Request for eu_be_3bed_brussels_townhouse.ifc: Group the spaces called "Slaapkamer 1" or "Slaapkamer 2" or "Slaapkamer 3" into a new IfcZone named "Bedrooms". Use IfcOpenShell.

First a look at what the model holds.

```python
import ifcopenshell

model = ifcopenshell.open("eu_be_3bed_brussels_townhouse.ifc")
print(model.schema)
seen = {}
for space in model.by_type("IfcSpace"):
    seen[space.LongName] = seen.get(space.LongName, 0) + 1
for name, count in sorted(seen.items(), key=str):
    print(count, "x", name)
print("zones:", [z.Name for z in model.by_type("IfcZone")][:20])
```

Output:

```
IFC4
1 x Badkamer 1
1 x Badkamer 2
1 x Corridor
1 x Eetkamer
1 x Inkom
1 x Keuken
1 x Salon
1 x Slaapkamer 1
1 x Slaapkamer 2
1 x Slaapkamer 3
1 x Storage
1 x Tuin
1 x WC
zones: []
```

```python
import ifcopenshell
import ifcopenshell.api.group
import ifcopenshell.api.root

model = ifcopenshell.open("eu_be_3bed_brussels_townhouse.ifc")

names = {"Slaapkamer 1", "Slaapkamer 2", "Slaapkamer 3"}
spaces = [s for s in model.by_type("IfcSpace") if s.LongName in names]

zone = ifcopenshell.api.root.create_entity(model, ifc_class="IfcZone", name="Bedrooms")
ifcopenshell.api.group.assign_group(model, products=spaces, group=zone)
print(len(spaces), "spaces in", zone.Name)

model.write("eu_be_3bed_brussels_townhouse_edited.ifc")
```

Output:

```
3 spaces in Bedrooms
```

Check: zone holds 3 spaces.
